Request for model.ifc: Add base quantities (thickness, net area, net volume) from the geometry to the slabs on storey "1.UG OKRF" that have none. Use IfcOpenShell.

First a look at what the model holds.

```python
import ifcopenshell
import ifcopenshell.util.element
import ifcopenshell.util.unit

model = ifcopenshell.open("model.ifc")
print(model.schema)
for unit_type in ("LENGTHUNIT", "AREAUNIT", "VOLUMEUNIT"):
    print(unit_type, ifcopenshell.util.unit.calculate_unit_scale(model, unit_type))
storey = next(s for s in model.by_type("IfcBuildingStorey") if s.Name == "1.UG OKRF")
slabs = [e for e in ifcopenshell.util.element.get_decomposition(storey) if e.is_a("IfcSlab")]
for e in sorted(slabs, key=lambda e: e.id()):
    print(e.id(), e.is_a(), e.Name, list(ifcopenshell.util.element.get_psets(e, qtos_only=True)), sep=" | ")
```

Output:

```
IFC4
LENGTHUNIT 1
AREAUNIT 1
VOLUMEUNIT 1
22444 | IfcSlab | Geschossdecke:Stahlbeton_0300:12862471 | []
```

```python
import ifcopenshell
import ifcopenshell.api.pset
import ifcopenshell.geom
import ifcopenshell.util.element
import ifcopenshell.util.shape
import ifcopenshell.util.unit

model = ifcopenshell.open("model.ifc")
unit_scale = ifcopenshell.util.unit.calculate_unit_scale(model)
area_scale = ifcopenshell.util.unit.calculate_unit_scale(model, "AREAUNIT")
volume_scale = ifcopenshell.util.unit.calculate_unit_scale(model, "VOLUMEUNIT")
settings = ifcopenshell.geom.settings()

storey = next(s for s in model.by_type("IfcBuildingStorey") if s.Name == "1.UG OKRF")
slabs = [e for e in ifcopenshell.util.element.get_decomposition(storey) if e.is_a("IfcSlab")]

for e in sorted(slabs, key=lambda e: e.id()):
    if ifcopenshell.util.element.get_psets(e, qtos_only=True, should_inherit=False):
        continue
    # Geometry comes back in metres, in the element's own axes.
    shape = ifcopenshell.geom.create_shape(settings, e)
    values = {
        "Width": ifcopenshell.util.shape.get_z(shape.geometry) / unit_scale,
        "NetArea": ifcopenshell.util.shape.get_footprint_area(shape.geometry) / area_scale,
        "NetVolume": ifcopenshell.util.shape.get_volume(shape.geometry) / volume_scale,
    }
    qto = ifcopenshell.api.pset.add_qto(model, product=e, name="Qto_SlabBaseQuantities")
    ifcopenshell.api.pset.edit_qto(model, qto=qto, properties=values)
    print(e.id(), {k: round(v, 3) for k, v in values.items()})

model.write("model_v2.ifc")
```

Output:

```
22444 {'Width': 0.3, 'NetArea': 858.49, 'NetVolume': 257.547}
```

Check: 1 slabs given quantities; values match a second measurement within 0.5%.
